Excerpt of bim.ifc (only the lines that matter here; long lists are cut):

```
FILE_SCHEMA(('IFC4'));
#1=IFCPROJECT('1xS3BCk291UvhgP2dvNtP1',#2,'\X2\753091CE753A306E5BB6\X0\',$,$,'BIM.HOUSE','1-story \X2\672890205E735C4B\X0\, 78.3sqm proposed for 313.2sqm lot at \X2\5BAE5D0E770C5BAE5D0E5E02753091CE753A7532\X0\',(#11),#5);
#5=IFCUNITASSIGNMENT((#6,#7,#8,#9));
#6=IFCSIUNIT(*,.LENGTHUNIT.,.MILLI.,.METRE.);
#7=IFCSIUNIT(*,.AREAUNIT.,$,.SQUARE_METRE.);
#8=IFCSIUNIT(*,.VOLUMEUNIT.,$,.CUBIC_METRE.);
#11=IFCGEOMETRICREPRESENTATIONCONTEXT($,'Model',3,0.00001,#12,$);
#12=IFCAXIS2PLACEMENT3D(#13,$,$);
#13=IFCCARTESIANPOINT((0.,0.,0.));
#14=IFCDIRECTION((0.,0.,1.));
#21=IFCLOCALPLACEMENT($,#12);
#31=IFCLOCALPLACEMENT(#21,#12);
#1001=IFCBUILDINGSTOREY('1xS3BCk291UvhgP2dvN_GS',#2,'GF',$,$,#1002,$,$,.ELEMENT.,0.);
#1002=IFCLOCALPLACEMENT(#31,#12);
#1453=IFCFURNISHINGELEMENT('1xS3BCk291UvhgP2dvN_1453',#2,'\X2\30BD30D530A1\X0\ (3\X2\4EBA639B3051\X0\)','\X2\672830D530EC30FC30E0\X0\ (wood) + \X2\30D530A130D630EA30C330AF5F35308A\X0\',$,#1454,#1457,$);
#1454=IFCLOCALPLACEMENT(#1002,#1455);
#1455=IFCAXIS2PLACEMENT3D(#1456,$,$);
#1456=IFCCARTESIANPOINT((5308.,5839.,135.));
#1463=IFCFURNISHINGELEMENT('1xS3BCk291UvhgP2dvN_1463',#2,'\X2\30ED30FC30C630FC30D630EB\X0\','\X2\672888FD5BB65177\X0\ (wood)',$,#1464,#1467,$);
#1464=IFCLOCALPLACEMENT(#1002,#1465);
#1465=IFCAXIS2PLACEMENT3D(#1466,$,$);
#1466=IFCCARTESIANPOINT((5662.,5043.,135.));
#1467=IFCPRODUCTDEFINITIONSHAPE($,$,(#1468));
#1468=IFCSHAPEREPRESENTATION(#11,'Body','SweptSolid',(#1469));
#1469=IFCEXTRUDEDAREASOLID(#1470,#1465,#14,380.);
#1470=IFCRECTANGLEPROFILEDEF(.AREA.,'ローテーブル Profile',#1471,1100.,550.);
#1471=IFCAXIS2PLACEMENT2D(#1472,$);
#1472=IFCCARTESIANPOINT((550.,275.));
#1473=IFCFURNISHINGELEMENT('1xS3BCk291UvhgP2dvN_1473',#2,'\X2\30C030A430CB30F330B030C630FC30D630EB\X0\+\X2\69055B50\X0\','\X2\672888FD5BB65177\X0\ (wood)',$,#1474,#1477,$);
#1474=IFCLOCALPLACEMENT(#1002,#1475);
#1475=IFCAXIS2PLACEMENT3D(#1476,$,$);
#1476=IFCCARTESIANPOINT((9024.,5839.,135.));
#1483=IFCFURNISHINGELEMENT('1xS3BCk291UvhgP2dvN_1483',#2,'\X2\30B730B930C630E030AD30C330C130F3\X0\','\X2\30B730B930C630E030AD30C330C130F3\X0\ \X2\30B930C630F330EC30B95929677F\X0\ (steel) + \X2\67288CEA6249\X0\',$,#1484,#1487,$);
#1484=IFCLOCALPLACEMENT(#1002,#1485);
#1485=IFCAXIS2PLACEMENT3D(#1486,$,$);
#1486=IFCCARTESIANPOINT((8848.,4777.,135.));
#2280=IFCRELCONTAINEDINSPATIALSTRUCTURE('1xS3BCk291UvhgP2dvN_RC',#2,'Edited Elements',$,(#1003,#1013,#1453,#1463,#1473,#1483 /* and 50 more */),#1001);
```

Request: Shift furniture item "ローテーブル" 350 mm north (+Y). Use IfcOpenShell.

```python
import ifcopenshell
import ifcopenshell.api.geometry
import ifcopenshell.util.placement
import ifcopenshell.util.unit

model = ifcopenshell.open("bim.ifc")
unit_scale = ifcopenshell.util.unit.calculate_unit_scale(model)

item = model.by_guid("1xS3BCk291UvhgP2dvN_1463")
matrix = ifcopenshell.util.placement.get_local_placement(item.ObjectPlacement)
matrix[1, 3] += 0.35 / unit_scale
ifcopenshell.api.geometry.edit_object_placement(model, product=item, matrix=matrix, is_si=False)

print(ifcopenshell.util.placement.get_local_placement(item.ObjectPlacement).round(3) + 0.0)

model.write("bim_rev.ifc")
```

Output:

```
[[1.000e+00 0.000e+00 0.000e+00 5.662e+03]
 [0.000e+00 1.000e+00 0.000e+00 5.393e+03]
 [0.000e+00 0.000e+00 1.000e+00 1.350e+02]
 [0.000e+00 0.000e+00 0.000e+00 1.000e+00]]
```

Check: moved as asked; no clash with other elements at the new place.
